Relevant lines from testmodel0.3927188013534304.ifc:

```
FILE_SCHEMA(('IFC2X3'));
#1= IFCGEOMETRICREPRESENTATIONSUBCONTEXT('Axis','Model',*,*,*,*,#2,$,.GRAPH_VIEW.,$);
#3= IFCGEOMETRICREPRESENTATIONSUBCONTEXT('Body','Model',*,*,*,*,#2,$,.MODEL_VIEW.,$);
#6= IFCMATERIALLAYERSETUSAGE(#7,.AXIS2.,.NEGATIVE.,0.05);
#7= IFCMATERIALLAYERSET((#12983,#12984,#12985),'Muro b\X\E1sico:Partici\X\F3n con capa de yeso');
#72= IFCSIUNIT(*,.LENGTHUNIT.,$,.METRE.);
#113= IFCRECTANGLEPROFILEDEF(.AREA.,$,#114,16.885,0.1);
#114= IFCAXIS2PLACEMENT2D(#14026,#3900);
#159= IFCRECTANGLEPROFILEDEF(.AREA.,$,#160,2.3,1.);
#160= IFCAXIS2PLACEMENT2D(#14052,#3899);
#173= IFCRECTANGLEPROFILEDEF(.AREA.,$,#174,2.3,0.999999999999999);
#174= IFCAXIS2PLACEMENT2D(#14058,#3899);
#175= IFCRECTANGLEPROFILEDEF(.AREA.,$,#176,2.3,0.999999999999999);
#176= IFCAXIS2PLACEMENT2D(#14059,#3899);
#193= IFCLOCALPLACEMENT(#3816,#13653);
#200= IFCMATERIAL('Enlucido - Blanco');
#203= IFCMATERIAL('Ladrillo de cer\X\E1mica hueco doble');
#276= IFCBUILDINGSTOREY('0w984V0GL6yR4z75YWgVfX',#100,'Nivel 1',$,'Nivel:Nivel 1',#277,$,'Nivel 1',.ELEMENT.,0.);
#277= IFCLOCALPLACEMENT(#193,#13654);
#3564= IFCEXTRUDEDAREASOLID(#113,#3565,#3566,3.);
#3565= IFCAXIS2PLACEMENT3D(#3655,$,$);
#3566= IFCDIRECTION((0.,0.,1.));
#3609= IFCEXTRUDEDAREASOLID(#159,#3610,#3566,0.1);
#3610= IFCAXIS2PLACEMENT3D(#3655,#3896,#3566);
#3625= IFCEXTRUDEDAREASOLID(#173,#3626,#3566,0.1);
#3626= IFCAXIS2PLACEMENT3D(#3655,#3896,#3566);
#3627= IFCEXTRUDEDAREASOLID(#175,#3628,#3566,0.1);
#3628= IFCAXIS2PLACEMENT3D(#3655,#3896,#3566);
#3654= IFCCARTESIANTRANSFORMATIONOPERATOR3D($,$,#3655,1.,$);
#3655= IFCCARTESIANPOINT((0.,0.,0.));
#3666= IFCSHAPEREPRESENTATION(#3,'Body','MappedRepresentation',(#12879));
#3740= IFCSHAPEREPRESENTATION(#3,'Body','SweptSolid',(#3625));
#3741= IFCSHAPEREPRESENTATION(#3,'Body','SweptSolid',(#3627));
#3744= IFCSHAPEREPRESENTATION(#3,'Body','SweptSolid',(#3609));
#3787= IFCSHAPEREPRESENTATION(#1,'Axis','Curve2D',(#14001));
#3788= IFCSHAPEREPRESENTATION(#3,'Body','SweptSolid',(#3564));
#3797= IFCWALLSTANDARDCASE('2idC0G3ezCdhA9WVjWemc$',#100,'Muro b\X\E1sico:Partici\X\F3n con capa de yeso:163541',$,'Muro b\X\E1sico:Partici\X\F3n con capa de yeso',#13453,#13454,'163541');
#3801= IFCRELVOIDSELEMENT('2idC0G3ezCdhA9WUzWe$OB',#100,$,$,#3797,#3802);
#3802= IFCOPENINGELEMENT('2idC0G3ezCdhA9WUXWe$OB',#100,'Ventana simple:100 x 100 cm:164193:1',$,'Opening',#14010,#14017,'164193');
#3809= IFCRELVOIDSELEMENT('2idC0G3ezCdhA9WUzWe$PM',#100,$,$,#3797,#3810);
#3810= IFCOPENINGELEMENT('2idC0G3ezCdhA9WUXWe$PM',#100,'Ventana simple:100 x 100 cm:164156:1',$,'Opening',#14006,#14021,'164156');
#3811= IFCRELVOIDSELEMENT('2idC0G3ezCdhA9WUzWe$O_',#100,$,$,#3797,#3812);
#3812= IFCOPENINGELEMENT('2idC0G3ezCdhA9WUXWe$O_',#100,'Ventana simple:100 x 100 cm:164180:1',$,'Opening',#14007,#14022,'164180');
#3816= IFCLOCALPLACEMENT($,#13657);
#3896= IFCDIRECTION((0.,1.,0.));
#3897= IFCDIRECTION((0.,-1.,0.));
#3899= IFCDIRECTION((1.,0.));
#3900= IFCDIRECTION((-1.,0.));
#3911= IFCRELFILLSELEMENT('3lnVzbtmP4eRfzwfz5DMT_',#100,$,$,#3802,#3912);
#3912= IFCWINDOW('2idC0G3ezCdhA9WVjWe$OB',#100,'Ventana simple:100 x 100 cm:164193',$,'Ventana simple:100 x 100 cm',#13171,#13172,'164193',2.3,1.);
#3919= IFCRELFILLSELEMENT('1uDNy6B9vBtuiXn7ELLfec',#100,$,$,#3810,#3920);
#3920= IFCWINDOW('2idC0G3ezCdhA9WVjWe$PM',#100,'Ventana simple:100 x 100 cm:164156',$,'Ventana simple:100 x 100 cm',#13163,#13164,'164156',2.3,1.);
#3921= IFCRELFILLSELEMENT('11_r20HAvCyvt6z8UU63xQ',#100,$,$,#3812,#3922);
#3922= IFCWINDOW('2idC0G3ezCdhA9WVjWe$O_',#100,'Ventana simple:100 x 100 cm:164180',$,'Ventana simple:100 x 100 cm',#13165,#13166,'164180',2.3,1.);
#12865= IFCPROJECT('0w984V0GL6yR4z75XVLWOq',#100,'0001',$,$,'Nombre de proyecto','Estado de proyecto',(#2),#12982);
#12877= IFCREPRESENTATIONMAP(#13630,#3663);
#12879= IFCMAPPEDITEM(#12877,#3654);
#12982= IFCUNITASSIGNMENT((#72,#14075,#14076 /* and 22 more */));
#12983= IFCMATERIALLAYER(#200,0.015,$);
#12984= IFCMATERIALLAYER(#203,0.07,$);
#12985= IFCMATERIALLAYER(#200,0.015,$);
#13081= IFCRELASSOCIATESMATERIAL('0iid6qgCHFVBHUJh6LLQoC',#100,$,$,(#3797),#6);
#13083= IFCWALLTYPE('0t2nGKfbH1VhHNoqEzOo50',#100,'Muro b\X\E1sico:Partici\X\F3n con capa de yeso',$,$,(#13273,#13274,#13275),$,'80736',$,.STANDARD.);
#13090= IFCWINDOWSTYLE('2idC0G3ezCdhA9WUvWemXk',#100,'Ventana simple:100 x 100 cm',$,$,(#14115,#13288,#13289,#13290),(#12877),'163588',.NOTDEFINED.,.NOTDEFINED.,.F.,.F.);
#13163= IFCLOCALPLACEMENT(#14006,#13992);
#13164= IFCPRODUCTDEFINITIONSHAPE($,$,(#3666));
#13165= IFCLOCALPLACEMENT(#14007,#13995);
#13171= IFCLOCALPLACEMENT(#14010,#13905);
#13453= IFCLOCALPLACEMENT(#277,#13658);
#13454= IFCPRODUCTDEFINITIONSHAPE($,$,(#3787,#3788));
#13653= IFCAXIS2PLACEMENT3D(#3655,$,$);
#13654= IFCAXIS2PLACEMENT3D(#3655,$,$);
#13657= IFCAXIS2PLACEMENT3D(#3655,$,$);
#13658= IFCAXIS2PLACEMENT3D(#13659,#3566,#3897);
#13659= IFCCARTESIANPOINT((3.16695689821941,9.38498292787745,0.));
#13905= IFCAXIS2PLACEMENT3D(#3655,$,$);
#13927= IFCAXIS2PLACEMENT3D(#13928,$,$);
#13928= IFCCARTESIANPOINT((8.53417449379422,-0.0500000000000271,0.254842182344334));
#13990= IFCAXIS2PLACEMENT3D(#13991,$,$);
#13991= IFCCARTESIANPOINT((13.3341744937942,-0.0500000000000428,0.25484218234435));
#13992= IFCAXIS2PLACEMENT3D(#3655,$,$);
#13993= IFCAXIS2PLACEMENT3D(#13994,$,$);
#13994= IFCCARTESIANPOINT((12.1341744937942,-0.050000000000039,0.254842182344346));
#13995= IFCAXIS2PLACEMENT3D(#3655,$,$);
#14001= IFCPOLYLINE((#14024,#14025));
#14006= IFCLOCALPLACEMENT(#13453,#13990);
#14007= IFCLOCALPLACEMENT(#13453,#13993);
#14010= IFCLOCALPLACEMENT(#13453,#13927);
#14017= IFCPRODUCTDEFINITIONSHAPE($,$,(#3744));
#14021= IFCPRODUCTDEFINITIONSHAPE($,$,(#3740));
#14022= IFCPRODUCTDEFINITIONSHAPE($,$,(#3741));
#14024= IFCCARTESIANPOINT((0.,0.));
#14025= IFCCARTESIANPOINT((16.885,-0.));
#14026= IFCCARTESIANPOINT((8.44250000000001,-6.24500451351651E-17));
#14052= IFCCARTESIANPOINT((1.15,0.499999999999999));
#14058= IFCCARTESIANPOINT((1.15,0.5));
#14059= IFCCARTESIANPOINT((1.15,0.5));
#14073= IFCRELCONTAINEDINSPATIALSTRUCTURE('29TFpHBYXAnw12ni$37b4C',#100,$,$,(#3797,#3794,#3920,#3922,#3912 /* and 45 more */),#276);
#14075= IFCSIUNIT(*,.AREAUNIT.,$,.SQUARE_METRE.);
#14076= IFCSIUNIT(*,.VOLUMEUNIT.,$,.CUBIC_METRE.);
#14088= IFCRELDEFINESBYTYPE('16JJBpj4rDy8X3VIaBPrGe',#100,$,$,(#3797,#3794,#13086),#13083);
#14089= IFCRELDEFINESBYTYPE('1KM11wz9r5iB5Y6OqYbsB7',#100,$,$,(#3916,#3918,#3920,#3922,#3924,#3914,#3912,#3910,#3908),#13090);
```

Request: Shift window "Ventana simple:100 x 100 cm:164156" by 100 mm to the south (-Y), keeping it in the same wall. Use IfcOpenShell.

```python
import ifcopenshell
import ifcopenshell.api.geometry
import ifcopenshell.util.placement
import ifcopenshell.util.unit

model = ifcopenshell.open("testmodel0.3927188013534304.ifc")
unit_scale = ifcopenshell.util.unit.calculate_unit_scale(model)

window = model.by_guid("2idC0G3ezCdhA9WVjWe$PM")
opening = window.FillsVoids[0].RelatingOpeningElement
wall = opening.VoidsElements[0].RelatingBuildingElement

wall_matrix = ifcopenshell.util.placement.get_local_placement(wall.ObjectPlacement)
shift = wall_matrix[:3, 0] * 0.1 / unit_scale
before = ifcopenshell.util.placement.get_local_placement(window.ObjectPlacement)[:3, 3].copy()

# The window is placed relative to its opening, so it follows when the opening moves.
matrix = ifcopenshell.util.placement.get_local_placement(opening.ObjectPlacement)
matrix[:3, 3] += shift
ifcopenshell.api.geometry.edit_object_placement(
    model, product=opening, matrix=matrix, is_si=False, should_transform_children=True
)

after = ifcopenshell.util.placement.get_local_placement(window.ObjectPlacement)[:3, 3]
print("window moved by", (after - before).round(3) + 0.0)

model.write("testmodel0.3927188013534304_edited.ifc")
```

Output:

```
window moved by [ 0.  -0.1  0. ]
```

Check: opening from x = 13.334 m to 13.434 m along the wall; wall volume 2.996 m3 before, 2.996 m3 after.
